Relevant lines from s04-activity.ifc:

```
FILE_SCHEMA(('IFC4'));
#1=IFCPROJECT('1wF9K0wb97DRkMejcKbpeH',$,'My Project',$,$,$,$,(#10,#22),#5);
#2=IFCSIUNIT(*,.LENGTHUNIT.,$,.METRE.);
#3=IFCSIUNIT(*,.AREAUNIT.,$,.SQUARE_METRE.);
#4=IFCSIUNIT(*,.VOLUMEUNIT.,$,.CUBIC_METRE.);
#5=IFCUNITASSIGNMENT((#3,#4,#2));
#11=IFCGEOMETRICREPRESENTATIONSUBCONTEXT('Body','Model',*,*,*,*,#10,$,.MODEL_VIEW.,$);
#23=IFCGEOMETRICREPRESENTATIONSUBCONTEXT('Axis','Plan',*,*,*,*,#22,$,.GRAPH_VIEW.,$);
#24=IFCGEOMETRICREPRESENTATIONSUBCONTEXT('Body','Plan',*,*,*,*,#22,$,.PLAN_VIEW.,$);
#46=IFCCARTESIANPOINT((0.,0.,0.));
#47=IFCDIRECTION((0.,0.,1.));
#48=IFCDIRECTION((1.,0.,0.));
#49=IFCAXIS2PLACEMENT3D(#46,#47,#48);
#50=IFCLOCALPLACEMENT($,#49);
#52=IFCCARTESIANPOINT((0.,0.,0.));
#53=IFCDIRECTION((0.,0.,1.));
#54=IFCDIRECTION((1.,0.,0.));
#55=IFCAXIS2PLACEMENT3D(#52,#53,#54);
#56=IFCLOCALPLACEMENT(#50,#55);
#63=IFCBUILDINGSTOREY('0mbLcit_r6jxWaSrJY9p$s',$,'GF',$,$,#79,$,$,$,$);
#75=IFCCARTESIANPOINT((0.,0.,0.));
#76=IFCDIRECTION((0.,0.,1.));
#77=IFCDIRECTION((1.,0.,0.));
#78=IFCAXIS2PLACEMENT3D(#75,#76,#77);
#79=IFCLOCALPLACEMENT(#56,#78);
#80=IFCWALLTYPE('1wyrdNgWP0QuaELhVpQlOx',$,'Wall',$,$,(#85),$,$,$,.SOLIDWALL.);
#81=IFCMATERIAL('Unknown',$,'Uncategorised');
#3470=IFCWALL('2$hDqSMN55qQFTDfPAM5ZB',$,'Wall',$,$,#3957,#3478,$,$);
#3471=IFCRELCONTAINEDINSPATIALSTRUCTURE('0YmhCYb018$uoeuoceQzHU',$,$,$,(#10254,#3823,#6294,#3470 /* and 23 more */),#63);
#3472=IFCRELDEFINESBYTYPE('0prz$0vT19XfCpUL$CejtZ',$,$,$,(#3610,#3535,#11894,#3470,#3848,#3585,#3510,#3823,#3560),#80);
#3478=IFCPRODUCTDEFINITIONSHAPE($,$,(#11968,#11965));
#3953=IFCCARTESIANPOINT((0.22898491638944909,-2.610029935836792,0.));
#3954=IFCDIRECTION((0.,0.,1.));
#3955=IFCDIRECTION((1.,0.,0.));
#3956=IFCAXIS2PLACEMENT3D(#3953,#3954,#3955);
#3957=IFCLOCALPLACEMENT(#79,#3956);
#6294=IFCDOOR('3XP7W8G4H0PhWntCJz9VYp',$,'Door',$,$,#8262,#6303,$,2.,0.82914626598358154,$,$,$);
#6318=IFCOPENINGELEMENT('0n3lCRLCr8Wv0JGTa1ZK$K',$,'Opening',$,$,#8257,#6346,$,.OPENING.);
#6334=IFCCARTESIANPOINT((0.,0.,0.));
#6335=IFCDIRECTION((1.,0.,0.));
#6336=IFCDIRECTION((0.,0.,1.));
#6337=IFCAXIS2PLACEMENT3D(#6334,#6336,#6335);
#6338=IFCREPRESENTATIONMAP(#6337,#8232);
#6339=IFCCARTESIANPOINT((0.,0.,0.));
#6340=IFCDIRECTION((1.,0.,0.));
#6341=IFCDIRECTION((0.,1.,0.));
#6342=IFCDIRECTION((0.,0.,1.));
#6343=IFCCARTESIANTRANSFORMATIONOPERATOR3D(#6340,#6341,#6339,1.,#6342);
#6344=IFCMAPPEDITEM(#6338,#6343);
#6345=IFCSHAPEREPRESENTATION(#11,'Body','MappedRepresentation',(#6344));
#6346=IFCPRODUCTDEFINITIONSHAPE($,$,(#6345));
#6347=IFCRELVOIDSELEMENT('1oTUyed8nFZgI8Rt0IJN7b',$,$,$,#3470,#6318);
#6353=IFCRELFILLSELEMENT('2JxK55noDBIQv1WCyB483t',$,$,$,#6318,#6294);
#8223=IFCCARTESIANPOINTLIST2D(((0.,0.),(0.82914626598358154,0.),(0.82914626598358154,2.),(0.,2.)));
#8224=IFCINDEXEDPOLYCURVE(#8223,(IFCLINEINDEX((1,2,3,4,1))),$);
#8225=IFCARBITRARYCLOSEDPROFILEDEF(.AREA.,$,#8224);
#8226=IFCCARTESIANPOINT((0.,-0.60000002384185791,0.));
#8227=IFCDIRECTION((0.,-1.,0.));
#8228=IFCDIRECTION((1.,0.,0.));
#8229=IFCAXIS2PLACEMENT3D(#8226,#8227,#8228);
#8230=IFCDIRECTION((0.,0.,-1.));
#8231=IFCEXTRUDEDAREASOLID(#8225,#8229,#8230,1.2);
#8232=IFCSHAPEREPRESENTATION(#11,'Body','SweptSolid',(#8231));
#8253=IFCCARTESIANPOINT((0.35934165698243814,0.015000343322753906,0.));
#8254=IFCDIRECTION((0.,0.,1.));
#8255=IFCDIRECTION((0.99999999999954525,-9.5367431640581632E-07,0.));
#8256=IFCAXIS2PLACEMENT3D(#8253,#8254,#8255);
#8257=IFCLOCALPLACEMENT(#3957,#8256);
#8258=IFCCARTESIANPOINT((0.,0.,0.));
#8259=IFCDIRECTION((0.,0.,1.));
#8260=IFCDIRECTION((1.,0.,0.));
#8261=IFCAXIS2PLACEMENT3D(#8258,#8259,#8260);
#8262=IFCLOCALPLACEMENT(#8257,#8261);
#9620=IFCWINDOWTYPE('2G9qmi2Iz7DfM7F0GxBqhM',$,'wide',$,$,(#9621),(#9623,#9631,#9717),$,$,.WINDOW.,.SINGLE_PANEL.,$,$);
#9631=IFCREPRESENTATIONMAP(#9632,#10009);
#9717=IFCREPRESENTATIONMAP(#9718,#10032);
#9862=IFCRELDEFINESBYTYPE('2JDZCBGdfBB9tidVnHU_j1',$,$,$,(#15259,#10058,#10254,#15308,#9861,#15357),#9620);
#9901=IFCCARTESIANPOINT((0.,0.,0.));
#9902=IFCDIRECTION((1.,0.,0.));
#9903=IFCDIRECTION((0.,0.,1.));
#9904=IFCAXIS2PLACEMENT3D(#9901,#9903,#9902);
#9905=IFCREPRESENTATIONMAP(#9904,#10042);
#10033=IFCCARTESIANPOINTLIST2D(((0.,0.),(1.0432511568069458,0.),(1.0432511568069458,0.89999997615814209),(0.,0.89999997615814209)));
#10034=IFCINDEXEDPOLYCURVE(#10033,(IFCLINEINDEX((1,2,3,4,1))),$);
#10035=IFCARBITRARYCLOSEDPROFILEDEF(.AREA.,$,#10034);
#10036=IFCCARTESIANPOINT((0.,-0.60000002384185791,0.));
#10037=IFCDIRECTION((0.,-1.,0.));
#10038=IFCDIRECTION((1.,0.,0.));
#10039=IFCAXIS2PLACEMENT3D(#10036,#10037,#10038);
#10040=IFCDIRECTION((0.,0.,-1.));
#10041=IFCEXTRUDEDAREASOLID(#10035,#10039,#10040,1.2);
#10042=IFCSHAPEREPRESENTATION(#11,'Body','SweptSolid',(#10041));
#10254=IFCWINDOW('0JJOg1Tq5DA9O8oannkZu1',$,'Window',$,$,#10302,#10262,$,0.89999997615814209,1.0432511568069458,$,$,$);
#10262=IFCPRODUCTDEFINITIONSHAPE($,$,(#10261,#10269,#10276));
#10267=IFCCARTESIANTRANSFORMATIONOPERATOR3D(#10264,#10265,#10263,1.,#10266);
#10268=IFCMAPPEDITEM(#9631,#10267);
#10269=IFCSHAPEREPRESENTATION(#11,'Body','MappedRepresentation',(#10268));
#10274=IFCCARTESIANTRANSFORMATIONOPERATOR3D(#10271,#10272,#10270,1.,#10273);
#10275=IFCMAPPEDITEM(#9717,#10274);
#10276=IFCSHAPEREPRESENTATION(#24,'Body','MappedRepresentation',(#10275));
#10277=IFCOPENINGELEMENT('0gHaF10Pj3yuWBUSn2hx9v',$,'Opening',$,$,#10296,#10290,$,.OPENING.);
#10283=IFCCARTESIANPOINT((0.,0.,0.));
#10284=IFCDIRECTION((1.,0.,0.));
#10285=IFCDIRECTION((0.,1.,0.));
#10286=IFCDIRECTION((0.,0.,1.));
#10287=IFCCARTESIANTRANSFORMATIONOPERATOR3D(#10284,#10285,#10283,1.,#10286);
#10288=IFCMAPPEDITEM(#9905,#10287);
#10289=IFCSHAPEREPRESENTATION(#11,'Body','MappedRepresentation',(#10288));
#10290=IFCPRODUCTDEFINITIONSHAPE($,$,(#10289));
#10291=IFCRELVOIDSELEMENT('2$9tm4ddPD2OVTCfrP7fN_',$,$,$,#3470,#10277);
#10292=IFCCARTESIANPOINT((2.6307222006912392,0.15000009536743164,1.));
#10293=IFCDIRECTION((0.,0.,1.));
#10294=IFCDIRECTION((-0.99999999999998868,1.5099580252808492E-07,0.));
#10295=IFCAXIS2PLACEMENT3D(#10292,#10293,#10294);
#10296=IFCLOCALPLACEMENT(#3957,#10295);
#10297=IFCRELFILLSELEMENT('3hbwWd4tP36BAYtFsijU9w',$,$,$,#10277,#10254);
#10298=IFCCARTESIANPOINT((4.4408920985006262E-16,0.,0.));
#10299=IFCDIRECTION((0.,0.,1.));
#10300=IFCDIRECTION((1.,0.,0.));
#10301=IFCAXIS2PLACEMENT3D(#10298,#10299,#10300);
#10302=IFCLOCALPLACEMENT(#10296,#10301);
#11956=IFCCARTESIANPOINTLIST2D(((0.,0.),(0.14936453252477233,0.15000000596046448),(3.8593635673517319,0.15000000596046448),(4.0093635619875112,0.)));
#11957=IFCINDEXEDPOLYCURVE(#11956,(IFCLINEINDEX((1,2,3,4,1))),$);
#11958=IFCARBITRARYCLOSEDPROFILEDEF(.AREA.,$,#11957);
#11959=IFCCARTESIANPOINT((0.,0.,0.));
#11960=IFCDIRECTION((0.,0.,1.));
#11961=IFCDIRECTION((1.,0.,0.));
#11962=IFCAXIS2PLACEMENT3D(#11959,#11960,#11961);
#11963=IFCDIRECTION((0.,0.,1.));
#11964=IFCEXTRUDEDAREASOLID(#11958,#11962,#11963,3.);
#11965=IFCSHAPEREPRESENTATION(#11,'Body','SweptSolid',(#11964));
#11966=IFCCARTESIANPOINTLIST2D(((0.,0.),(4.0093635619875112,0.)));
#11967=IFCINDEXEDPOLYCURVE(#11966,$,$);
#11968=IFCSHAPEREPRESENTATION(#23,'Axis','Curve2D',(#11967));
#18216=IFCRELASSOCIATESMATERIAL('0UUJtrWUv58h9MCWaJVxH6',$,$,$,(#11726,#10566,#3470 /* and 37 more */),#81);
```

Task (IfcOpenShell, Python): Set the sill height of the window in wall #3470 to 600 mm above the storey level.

```python
import numpy as np
import ifcopenshell
import ifcopenshell.api.geometry
import ifcopenshell.geom
import ifcopenshell.util.element
import ifcopenshell.util.placement
import ifcopenshell.util.shape
import ifcopenshell.util.unit

model = ifcopenshell.open("s04-activity.ifc")
unit_scale = ifcopenshell.util.unit.calculate_unit_scale(model)

window = model.by_guid("0JJOg1Tq5DA9O8oannkZu1")
opening = window.FillsVoids[0].RelatingOpeningElement
storey = ifcopenshell.util.element.get_container(window, ifc_class="IfcBuildingStorey")
level = ifcopenshell.util.placement.get_local_placement(storey.ObjectPlacement)[2, 3]

# The opening's origin need not be at the sill, so measure its lowest point.
shape = ifcopenshell.geom.create_shape(ifcopenshell.geom.settings(), opening)
bottom = ifcopenshell.util.shape.get_shape_bottom_elevation(shape, shape.geometry) / unit_scale
dz = level + 0.6 / unit_scale - bottom

shift = np.array([0.0, 0.0, dz])
# The window is placed relative to its opening, so it follows when the opening moves.
matrix = ifcopenshell.util.placement.get_local_placement(opening.ObjectPlacement)
matrix[:3, 3] += shift
ifcopenshell.api.geometry.edit_object_placement(
    model, product=opening, matrix=matrix, is_si=False, should_transform_children=True
)

print(f"moved by {dz * unit_scale:+.3f} m")

model.write("s04-activity_v2.ifc")
```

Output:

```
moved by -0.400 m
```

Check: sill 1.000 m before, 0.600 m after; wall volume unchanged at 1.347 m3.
